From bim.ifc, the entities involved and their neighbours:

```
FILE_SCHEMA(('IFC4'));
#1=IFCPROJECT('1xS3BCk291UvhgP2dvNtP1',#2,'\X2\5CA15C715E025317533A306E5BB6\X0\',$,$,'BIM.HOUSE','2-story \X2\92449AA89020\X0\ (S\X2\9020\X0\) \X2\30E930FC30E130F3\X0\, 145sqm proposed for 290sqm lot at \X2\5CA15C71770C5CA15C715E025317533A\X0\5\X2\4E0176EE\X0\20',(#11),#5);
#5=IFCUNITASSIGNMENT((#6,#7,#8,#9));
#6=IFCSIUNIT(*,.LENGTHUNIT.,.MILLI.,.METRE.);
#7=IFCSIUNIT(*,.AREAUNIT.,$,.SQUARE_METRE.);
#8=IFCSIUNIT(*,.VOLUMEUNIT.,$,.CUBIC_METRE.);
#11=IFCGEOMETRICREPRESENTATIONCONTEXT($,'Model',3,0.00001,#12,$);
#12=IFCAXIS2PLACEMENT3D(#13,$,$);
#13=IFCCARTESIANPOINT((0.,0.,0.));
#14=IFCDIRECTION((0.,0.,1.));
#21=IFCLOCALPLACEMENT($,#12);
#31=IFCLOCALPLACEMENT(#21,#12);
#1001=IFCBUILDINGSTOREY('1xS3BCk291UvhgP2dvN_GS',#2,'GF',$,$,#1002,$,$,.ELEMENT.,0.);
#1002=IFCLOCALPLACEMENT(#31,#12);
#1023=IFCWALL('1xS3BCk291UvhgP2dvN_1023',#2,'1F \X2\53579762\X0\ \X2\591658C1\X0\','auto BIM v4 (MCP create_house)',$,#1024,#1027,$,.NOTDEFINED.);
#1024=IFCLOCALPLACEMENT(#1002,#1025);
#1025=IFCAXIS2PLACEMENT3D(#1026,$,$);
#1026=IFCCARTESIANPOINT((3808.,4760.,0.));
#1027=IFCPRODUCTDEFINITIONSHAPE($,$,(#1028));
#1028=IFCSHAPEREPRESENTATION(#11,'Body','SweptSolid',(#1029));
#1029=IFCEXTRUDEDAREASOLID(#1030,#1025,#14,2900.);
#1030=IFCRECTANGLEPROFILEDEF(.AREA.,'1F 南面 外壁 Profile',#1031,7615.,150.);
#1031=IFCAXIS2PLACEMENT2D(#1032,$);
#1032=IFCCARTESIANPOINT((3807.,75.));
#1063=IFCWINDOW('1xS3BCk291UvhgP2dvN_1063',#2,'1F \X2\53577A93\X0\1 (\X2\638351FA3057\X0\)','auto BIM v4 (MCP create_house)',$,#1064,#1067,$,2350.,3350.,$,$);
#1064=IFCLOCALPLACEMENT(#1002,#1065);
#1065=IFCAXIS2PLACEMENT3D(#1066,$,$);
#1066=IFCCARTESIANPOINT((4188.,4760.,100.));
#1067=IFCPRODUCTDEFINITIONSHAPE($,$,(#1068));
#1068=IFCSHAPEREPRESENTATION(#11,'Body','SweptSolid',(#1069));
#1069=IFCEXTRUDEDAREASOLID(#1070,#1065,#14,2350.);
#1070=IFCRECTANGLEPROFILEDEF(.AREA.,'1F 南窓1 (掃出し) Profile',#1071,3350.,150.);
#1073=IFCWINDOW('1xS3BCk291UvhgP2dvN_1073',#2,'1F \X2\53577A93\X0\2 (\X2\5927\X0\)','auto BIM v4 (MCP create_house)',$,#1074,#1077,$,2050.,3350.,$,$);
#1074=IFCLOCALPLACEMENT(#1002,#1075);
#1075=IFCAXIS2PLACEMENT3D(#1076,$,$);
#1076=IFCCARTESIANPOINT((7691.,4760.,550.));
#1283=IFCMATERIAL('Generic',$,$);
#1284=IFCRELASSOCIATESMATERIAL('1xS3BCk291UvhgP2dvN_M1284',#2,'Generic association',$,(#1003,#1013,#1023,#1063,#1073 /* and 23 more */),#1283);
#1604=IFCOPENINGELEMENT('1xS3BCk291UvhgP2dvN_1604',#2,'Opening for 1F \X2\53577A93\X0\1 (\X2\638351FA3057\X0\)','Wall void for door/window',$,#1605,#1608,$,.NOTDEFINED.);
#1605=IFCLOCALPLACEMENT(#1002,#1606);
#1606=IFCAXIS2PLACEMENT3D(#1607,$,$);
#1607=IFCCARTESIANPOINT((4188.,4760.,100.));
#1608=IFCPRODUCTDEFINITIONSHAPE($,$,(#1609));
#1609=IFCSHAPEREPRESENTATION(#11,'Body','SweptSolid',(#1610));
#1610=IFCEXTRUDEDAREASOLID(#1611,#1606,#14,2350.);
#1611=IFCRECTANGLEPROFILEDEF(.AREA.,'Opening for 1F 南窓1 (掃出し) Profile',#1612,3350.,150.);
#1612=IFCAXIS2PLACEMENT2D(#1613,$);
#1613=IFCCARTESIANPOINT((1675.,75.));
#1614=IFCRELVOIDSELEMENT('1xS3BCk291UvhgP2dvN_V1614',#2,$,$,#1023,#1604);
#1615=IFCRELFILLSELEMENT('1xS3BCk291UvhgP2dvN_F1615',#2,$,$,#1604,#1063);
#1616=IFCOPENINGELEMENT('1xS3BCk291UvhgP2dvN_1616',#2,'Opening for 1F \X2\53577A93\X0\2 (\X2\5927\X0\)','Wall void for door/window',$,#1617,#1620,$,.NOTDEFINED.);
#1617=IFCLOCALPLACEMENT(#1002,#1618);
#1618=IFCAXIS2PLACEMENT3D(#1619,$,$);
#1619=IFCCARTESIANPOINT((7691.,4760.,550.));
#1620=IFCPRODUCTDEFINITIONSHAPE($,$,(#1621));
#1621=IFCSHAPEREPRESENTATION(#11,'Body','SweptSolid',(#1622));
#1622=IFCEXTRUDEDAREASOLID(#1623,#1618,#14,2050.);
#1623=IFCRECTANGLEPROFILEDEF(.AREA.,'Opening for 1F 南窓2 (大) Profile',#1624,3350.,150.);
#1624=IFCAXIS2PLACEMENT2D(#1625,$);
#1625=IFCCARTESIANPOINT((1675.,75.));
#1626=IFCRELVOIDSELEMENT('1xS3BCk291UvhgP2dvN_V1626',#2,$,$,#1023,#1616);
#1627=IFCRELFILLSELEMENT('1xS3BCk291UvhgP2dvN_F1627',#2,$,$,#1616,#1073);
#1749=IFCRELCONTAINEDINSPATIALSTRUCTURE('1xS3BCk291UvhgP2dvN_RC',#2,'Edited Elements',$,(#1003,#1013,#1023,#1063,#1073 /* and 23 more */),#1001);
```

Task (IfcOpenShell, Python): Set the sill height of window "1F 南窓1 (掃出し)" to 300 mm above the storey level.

```python
import numpy as np
import ifcopenshell
import ifcopenshell.api.geometry
import ifcopenshell.geom
import ifcopenshell.util.element
import ifcopenshell.util.placement
import ifcopenshell.util.shape
import ifcopenshell.util.unit

model = ifcopenshell.open("bim.ifc")
unit_scale = ifcopenshell.util.unit.calculate_unit_scale(model)

window = model.by_id(1063)
opening = window.FillsVoids[0].RelatingOpeningElement
storey = ifcopenshell.util.element.get_container(window, ifc_class="IfcBuildingStorey")
level = ifcopenshell.util.placement.get_local_placement(storey.ObjectPlacement)[2, 3]

# The opening's origin need not be at the sill, so measure its lowest point.
shape = ifcopenshell.geom.create_shape(ifcopenshell.geom.settings(), opening)
bottom = ifcopenshell.util.shape.get_shape_bottom_elevation(shape, shape.geometry) / unit_scale
dz = level + 300.0 - bottom

shift = np.array([0.0, 0.0, dz])
# The window is not placed relative to its opening, so move both.
for product in (opening, window):
    matrix = ifcopenshell.util.placement.get_local_placement(product.ObjectPlacement)
    matrix[:3, 3] += shift
    ifcopenshell.api.geometry.edit_object_placement(model, product=product, matrix=matrix, is_si=False)

print(f"moved by {dz * unit_scale:+.3f} m")

model.write("bim_v2.ifc")
```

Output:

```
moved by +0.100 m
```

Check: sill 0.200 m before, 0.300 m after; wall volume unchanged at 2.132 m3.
